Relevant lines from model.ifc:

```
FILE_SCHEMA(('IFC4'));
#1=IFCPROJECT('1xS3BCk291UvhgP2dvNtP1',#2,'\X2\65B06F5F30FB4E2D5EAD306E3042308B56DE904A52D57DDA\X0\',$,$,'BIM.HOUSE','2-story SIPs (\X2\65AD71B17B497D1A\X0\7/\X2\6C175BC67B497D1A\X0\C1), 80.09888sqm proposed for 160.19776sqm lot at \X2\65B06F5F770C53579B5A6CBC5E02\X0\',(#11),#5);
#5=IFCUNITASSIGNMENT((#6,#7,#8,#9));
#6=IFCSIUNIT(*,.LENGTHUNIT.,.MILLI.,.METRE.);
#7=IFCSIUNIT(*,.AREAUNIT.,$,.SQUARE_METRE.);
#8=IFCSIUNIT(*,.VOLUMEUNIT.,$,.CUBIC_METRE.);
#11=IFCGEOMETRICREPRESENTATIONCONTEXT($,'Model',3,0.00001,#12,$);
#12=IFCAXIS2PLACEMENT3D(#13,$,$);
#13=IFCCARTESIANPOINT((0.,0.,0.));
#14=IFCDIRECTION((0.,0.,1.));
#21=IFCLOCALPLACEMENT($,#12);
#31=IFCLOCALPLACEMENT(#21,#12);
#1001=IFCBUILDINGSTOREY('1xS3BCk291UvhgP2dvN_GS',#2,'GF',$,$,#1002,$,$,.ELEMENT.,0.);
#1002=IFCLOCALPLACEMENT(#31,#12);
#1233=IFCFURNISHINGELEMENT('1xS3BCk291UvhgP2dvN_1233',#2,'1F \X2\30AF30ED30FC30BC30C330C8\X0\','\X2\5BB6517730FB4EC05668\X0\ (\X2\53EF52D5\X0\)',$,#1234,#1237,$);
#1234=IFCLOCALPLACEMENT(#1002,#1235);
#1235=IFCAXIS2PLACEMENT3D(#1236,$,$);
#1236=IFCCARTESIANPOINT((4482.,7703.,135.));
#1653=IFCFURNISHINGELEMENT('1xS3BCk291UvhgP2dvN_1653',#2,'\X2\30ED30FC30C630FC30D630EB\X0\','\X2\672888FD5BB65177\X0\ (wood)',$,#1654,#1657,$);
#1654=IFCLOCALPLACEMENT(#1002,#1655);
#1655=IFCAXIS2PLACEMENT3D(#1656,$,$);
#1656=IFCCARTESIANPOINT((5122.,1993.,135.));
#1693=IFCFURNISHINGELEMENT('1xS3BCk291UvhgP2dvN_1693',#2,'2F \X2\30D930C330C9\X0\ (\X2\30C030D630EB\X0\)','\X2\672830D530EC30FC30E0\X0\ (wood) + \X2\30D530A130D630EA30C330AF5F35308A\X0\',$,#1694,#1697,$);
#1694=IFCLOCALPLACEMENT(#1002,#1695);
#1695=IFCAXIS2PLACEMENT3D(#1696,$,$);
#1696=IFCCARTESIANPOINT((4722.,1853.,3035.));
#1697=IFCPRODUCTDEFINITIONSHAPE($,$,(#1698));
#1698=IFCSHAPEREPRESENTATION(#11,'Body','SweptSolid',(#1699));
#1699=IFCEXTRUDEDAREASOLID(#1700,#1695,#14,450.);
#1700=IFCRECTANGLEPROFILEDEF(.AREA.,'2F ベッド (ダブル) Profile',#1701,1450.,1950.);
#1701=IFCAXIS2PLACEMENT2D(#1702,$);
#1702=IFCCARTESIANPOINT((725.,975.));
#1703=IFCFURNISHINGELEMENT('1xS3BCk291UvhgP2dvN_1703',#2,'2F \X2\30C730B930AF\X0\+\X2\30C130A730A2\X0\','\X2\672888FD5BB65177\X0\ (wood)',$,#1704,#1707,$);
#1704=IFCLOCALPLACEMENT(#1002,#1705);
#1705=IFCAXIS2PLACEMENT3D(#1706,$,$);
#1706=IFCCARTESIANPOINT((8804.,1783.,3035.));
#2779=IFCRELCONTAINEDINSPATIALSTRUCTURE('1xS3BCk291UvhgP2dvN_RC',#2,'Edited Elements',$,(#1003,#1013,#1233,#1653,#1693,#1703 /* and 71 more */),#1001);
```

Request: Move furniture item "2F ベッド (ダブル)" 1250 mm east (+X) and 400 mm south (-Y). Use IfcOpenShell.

```python
import ifcopenshell
import ifcopenshell.api.geometry
import ifcopenshell.util.placement
import ifcopenshell.util.unit

model = ifcopenshell.open("model.ifc")
unit_scale = ifcopenshell.util.unit.calculate_unit_scale(model)

item = model.by_guid("1xS3BCk291UvhgP2dvN_1693")
matrix = ifcopenshell.util.placement.get_local_placement(item.ObjectPlacement)
matrix[0, 3] += 1.25 / unit_scale
matrix[1, 3] -= 0.4 / unit_scale
ifcopenshell.api.geometry.edit_object_placement(model, product=item, matrix=matrix, is_si=False)

print(ifcopenshell.util.placement.get_local_placement(item.ObjectPlacement).round(3) + 0.0)

model.write("model_updated.ifc")
```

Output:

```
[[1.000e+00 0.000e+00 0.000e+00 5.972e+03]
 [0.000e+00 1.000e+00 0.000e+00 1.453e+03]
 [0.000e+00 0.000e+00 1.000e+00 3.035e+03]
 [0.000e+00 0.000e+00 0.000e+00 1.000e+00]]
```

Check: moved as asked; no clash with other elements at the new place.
